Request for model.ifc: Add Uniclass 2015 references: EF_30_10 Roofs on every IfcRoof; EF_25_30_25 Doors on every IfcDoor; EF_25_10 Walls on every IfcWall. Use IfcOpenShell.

First a look at what the model holds.

```python
import ifcopenshell

model = ifcopenshell.open("model.ifc")
print(model.schema)
print("classifications:", [c.Name for c in model.by_type("IfcClassification")])
for ifc_class in ("IfcDoor", "IfcRoof", "IfcStair", "IfcWall", "IfcWindow"):
    print(ifc_class, len(model.by_type(ifc_class)))
```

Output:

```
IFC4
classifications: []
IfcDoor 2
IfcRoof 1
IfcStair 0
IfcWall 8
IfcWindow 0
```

```python
import ifcopenshell
import ifcopenshell.api.classification

model = ifcopenshell.open("model.ifc")

system = ifcopenshell.api.classification.add_classification(model, classification="Uniclass 2015")

codes = {
    "IfcRoof": ("EF_30_10", "Roofs"),
    "IfcDoor": ("EF_25_30_25", "Doors"),
    "IfcWall": ("EF_25_10", "Walls"),
}
for ifc_class, (code, name) in codes.items():
    products = model.by_type(ifc_class)
    ifcopenshell.api.classification.add_reference(
        model, products=products, classification=system, identification=code, name=name
    )
    print(code, len(products))

model.write("model_updated.ifc")
```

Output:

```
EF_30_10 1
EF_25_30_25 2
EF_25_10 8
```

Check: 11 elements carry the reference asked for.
